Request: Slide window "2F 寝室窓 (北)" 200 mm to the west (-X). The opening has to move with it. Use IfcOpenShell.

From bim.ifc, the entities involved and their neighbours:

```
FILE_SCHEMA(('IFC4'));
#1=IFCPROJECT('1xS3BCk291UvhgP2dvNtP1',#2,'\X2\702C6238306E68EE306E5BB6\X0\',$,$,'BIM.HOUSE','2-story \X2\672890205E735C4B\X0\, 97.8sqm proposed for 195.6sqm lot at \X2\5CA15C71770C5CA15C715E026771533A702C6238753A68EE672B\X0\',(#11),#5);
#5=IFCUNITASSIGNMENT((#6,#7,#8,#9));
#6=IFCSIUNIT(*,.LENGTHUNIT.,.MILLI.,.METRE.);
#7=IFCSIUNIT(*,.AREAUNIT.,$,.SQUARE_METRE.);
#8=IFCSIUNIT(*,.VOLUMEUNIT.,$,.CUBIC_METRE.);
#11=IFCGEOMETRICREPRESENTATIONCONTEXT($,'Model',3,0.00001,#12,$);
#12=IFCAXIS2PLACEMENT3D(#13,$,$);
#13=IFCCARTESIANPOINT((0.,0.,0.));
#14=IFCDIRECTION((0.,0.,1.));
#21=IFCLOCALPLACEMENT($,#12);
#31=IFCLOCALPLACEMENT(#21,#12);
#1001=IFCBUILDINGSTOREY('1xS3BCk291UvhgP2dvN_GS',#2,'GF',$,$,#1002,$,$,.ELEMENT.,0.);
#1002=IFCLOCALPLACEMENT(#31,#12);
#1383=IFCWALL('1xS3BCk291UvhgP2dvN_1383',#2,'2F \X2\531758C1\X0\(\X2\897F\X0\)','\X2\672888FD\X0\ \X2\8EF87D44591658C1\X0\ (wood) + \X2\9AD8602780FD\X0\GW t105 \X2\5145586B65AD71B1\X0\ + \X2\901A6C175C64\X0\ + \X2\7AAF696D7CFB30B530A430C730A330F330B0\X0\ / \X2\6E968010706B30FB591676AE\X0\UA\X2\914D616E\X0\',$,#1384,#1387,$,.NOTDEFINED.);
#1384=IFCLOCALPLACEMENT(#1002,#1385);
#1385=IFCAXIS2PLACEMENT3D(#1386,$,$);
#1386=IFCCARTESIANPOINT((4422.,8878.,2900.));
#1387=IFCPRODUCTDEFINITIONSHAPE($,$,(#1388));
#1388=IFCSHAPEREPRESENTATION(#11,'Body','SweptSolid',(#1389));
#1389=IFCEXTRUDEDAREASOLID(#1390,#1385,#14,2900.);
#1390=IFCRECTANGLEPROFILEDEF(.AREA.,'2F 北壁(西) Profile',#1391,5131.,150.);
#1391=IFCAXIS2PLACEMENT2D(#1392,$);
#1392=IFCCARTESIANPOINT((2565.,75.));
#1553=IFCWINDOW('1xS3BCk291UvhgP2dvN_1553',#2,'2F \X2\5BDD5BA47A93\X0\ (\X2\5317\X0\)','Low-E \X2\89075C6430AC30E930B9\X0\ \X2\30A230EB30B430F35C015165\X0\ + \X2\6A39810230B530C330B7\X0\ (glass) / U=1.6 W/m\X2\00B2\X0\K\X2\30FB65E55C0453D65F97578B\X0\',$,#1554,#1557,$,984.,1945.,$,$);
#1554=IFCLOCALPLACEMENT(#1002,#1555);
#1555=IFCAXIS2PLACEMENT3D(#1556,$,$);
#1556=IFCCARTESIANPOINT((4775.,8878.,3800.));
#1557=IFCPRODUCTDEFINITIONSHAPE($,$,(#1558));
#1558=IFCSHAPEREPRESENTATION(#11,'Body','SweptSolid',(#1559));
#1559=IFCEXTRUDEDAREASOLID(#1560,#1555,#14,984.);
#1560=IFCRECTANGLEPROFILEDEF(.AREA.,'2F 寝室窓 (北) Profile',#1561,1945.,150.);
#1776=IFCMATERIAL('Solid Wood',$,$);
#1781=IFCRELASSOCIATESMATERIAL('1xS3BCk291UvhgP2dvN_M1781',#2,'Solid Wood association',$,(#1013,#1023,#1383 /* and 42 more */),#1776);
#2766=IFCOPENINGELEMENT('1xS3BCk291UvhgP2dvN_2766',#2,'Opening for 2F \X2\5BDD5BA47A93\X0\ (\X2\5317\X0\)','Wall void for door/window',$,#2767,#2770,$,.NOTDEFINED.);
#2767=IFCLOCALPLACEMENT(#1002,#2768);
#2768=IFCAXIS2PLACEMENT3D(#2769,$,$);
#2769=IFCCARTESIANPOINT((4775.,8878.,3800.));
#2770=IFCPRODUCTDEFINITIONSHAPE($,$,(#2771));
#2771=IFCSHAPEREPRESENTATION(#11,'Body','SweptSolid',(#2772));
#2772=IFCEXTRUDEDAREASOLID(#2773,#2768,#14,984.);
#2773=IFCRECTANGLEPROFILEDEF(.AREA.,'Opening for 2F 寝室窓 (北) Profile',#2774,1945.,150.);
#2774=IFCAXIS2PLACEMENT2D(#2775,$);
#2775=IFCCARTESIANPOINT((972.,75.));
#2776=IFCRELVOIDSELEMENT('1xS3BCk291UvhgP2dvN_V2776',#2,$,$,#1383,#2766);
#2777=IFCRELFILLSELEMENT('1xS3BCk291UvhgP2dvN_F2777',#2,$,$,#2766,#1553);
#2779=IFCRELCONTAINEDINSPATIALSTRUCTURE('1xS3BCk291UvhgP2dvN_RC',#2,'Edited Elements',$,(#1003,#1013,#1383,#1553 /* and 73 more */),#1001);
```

```python
import ifcopenshell
import ifcopenshell.api.geometry
import ifcopenshell.util.placement

model = ifcopenshell.open("bim.ifc")

window = model.by_id(1553)
opening = window.FillsVoids[0].RelatingOpeningElement
wall = opening.VoidsElements[0].RelatingBuildingElement

wall_matrix = ifcopenshell.util.placement.get_local_placement(wall.ObjectPlacement)
shift = wall_matrix[:3, 0] * -200.0
before = ifcopenshell.util.placement.get_local_placement(window.ObjectPlacement)[:3, 3].copy()

# The window is not placed relative to its opening, so move both.
for product in (opening, window):
    matrix = ifcopenshell.util.placement.get_local_placement(product.ObjectPlacement)
    matrix[:3, 3] += shift
    ifcopenshell.api.geometry.edit_object_placement(model, product=product, matrix=matrix, is_si=False)

after = ifcopenshell.util.placement.get_local_placement(window.ObjectPlacement)[:3, 3]
print("window moved by", (after - before).round(3) + 0.0)

model.write("bim_updated.ifc")
```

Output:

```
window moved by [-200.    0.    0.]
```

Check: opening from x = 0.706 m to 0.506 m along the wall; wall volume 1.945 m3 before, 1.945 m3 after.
